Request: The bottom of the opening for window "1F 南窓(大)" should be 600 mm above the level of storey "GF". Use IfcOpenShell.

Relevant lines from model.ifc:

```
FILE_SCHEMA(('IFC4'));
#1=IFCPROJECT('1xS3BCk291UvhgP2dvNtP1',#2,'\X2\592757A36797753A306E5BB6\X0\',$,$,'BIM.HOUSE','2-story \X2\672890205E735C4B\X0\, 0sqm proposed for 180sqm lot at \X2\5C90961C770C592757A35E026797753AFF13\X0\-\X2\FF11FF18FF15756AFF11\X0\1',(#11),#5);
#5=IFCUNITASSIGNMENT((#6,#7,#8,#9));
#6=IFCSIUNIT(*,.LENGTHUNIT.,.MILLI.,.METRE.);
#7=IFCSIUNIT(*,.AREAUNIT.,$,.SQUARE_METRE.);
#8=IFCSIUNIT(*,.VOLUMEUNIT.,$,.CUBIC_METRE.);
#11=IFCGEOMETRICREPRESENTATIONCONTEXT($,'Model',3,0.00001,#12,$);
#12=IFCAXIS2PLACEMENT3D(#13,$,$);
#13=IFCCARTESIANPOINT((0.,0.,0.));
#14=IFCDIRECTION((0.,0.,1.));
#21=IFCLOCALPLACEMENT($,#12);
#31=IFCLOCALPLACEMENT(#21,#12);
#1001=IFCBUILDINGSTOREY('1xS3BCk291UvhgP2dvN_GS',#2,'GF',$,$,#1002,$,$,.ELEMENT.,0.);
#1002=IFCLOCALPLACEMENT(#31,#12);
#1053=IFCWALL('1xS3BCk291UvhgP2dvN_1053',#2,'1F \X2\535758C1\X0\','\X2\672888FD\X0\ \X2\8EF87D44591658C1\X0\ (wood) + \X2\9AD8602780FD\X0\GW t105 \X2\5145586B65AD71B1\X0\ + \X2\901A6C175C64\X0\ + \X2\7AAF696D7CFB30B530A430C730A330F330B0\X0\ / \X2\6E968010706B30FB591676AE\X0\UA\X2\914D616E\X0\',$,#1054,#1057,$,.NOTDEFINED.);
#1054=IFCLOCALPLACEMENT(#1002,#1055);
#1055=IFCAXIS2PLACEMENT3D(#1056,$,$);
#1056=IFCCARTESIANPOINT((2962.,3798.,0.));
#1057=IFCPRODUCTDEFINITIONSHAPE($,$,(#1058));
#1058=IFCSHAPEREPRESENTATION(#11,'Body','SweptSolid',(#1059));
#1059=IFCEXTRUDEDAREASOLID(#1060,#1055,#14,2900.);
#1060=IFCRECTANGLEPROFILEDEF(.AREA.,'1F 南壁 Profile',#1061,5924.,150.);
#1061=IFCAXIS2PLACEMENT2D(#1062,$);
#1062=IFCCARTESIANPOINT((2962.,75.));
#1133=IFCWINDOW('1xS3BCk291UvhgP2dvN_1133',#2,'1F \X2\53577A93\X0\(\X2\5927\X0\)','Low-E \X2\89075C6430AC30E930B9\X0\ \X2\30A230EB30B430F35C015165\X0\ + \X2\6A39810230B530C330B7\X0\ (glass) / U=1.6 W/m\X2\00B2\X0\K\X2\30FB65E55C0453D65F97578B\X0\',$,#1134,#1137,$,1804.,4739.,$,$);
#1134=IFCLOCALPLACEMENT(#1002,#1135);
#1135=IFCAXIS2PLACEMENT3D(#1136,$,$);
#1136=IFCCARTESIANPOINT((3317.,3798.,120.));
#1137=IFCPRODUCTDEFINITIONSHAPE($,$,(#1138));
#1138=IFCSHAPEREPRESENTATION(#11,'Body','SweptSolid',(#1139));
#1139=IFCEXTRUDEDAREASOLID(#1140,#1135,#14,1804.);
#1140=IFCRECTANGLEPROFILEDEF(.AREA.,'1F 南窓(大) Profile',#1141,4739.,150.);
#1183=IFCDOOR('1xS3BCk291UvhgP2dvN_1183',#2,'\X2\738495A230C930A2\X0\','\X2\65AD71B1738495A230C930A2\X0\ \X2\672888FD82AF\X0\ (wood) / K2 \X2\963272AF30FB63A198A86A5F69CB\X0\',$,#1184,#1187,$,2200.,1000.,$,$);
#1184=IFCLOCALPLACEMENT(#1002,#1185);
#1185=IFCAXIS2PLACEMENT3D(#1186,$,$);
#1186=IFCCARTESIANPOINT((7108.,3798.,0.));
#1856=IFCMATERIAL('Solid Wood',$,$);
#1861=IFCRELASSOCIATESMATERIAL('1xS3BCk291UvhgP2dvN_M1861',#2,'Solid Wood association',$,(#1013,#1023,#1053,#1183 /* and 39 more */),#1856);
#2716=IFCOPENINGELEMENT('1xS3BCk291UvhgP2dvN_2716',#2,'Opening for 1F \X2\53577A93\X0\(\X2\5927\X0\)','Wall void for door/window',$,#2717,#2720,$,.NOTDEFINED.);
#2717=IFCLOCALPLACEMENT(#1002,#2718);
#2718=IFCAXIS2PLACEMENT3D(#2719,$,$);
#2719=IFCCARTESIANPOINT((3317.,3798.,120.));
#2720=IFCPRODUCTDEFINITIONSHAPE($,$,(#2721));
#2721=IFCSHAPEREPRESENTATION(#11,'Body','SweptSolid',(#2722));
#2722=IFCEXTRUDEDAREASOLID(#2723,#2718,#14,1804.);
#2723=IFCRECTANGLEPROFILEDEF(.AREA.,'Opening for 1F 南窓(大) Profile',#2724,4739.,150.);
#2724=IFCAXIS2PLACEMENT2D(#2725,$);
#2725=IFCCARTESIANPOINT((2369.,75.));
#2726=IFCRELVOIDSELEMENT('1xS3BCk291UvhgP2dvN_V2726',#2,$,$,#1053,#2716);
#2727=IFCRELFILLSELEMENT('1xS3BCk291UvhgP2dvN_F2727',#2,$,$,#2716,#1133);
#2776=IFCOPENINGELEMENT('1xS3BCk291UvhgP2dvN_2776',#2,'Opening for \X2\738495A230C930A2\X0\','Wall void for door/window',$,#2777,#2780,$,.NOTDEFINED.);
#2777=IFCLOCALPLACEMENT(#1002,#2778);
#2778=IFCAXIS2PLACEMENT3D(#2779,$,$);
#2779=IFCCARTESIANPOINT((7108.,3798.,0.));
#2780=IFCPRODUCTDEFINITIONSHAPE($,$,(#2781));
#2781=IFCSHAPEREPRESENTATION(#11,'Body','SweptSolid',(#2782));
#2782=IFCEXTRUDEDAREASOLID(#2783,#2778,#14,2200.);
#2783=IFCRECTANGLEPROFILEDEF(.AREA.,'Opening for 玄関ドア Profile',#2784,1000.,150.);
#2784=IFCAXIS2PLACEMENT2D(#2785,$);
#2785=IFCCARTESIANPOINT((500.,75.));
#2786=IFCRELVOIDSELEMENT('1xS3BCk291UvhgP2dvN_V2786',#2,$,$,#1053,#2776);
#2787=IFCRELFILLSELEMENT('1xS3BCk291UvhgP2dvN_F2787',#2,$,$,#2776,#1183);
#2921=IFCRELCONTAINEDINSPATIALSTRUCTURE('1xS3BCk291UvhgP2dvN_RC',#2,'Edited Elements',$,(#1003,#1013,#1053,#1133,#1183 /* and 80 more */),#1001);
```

```python
import numpy as np
import ifcopenshell
import ifcopenshell.api.geometry
import ifcopenshell.geom
import ifcopenshell.util.element
import ifcopenshell.util.placement
import ifcopenshell.util.shape
import ifcopenshell.util.unit

model = ifcopenshell.open("model.ifc")
unit_scale = ifcopenshell.util.unit.calculate_unit_scale(model)

window = model.by_guid("1xS3BCk291UvhgP2dvN_1133")
opening = window.FillsVoids[0].RelatingOpeningElement
storey = ifcopenshell.util.element.get_container(window, ifc_class="IfcBuildingStorey")
level = ifcopenshell.util.placement.get_local_placement(storey.ObjectPlacement)[2, 3]

# The opening's origin need not be at the sill, so measure its lowest point.
shape = ifcopenshell.geom.create_shape(ifcopenshell.geom.settings(), opening)
bottom = ifcopenshell.util.shape.get_shape_bottom_elevation(shape, shape.geometry) / unit_scale
dz = level + 0.6 / unit_scale - bottom

shift = np.array([0.0, 0.0, dz])
# The window is not placed relative to its opening, so move both.
for product in (opening, window):
    matrix = ifcopenshell.util.placement.get_local_placement(product.ObjectPlacement)
    matrix[:3, 3] += shift
    ifcopenshell.api.geometry.edit_object_placement(model, product=product, matrix=matrix, is_si=False)

print(f"moved by {dz * unit_scale:+.3f} m")

model.write("model_v2.ifc")
```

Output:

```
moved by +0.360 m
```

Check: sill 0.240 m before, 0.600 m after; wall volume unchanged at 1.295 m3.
